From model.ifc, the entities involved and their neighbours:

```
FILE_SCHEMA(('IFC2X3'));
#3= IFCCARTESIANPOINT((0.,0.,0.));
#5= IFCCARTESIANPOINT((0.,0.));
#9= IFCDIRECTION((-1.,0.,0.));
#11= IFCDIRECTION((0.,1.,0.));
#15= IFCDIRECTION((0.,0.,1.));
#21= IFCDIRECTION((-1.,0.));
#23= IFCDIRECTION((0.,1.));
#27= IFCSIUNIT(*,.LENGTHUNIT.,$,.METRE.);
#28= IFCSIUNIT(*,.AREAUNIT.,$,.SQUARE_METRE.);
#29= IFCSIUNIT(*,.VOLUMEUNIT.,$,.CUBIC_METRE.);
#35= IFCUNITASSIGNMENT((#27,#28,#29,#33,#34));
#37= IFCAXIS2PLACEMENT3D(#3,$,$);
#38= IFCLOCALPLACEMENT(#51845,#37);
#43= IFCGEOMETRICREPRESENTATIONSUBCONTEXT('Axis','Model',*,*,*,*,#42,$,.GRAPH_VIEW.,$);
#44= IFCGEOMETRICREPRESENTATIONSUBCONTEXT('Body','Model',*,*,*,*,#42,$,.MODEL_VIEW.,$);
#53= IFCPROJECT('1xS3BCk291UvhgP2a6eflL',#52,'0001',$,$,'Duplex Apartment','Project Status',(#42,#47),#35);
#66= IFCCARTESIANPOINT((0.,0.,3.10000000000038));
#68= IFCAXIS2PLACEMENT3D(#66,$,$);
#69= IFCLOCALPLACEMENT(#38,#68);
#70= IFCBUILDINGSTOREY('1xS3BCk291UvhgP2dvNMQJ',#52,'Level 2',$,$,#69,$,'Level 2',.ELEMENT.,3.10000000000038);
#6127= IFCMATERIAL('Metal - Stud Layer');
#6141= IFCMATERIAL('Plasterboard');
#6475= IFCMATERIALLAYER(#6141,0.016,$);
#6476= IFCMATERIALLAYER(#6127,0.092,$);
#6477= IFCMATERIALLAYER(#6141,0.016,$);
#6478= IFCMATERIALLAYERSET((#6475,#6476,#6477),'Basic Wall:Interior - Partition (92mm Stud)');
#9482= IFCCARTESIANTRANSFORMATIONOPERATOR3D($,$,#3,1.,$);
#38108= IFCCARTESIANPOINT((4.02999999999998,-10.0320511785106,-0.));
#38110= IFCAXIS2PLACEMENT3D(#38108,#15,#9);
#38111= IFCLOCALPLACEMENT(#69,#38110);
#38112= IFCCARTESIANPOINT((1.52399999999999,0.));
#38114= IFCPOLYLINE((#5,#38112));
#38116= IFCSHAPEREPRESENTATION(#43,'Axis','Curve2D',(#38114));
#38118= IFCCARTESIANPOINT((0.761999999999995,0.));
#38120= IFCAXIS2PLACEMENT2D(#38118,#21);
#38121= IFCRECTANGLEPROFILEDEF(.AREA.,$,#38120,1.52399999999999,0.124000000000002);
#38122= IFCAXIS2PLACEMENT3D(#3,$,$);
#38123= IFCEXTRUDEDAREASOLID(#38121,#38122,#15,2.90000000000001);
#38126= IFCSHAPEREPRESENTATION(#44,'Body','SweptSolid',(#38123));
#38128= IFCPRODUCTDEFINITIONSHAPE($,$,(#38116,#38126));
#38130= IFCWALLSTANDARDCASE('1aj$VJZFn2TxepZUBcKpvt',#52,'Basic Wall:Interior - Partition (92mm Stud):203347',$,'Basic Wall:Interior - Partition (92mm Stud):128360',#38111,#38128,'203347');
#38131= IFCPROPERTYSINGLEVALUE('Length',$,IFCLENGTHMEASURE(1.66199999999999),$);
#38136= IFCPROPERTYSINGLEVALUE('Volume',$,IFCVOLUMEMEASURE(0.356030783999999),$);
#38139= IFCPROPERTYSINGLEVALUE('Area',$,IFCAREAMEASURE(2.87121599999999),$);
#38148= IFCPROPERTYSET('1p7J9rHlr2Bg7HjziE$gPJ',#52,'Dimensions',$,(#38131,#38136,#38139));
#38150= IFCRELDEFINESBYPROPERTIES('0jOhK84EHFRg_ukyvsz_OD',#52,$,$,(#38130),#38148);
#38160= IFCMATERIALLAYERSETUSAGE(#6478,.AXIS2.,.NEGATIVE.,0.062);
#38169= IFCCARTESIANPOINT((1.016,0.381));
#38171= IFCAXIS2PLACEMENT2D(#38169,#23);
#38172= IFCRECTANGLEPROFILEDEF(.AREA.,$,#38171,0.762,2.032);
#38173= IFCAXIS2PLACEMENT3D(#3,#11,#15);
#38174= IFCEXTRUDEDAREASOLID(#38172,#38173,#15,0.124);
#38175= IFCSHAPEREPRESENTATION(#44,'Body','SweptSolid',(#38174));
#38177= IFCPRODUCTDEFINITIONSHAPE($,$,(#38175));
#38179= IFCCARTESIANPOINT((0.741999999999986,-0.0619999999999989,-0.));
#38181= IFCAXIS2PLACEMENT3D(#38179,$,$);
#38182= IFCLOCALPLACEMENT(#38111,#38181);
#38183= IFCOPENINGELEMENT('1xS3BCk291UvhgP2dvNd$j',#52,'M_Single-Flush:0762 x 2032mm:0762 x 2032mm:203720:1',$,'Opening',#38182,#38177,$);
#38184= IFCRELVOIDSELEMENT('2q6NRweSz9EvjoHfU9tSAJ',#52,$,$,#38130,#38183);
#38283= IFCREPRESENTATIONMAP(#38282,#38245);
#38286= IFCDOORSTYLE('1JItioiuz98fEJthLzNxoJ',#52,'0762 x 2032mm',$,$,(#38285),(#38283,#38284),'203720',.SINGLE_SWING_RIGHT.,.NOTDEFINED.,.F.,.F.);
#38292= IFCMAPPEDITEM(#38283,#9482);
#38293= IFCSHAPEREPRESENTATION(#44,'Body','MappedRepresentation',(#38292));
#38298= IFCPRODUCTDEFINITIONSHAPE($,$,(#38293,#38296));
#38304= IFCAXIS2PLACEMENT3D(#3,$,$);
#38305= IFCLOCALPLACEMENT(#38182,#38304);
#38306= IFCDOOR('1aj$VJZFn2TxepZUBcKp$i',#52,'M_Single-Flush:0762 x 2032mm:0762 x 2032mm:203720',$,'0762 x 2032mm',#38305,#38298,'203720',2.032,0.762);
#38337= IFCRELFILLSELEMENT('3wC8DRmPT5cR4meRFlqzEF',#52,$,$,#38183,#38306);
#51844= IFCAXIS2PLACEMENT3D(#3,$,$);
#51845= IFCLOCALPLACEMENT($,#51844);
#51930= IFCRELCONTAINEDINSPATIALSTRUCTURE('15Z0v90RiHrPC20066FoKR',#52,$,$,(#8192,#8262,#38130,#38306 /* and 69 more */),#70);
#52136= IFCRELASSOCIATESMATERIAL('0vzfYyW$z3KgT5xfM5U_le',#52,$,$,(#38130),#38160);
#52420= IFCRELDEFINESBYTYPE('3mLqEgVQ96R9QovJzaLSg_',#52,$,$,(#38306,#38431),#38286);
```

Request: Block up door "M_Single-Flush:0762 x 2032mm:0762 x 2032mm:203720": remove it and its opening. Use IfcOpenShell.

```python
import ifcopenshell
import ifcopenshell.api.feature
import ifcopenshell.api.pset
import ifcopenshell.api.root
import ifcopenshell.geom
import ifcopenshell.util.element
import ifcopenshell.util.shape
import ifcopenshell.util.unit

model = ifcopenshell.open("model.ifc")
area_scale = ifcopenshell.util.unit.calculate_unit_scale(model, "AREAUNIT")
volume_scale = ifcopenshell.util.unit.calculate_unit_scale(model, "VOLUMEUNIT")
settings = ifcopenshell.geom.settings()


def volume(element):
    """Net volume in cubic metres, openings subtracted."""
    shape = ifcopenshell.geom.create_shape(settings, element)
    return ifcopenshell.util.shape.get_volume(shape.geometry)


door = model.by_id(38306)
opening = door.FillsVoids[0].RelatingOpeningElement
wall = opening.VoidsElements[0].RelatingBuildingElement
before = volume(wall)

ifcopenshell.api.root.remove_product(model, product=door)
ifcopenshell.api.feature.remove_feature(model, feature=opening)

after = volume(wall)
thickness = 0.124  # wall thickness in metres

# Update the wall's stored quantities.
pset = model.by_id(ifcopenshell.util.element.get_pset(wall, "Dimensions", should_inherit=False)["id"])
ifcopenshell.api.pset.edit_pset(model, pset=pset, properties={
    "Volume": model.create_entity("IfcVolumeMeasure", after / volume_scale),
    "Area": model.create_entity("IfcAreaMeasure", after / thickness / area_scale),
})

print(f"wall volume {before:.3f} -> {after:.3f} m3")

model.write("model_edited.ifc")
```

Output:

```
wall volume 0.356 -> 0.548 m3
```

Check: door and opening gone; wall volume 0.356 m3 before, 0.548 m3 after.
